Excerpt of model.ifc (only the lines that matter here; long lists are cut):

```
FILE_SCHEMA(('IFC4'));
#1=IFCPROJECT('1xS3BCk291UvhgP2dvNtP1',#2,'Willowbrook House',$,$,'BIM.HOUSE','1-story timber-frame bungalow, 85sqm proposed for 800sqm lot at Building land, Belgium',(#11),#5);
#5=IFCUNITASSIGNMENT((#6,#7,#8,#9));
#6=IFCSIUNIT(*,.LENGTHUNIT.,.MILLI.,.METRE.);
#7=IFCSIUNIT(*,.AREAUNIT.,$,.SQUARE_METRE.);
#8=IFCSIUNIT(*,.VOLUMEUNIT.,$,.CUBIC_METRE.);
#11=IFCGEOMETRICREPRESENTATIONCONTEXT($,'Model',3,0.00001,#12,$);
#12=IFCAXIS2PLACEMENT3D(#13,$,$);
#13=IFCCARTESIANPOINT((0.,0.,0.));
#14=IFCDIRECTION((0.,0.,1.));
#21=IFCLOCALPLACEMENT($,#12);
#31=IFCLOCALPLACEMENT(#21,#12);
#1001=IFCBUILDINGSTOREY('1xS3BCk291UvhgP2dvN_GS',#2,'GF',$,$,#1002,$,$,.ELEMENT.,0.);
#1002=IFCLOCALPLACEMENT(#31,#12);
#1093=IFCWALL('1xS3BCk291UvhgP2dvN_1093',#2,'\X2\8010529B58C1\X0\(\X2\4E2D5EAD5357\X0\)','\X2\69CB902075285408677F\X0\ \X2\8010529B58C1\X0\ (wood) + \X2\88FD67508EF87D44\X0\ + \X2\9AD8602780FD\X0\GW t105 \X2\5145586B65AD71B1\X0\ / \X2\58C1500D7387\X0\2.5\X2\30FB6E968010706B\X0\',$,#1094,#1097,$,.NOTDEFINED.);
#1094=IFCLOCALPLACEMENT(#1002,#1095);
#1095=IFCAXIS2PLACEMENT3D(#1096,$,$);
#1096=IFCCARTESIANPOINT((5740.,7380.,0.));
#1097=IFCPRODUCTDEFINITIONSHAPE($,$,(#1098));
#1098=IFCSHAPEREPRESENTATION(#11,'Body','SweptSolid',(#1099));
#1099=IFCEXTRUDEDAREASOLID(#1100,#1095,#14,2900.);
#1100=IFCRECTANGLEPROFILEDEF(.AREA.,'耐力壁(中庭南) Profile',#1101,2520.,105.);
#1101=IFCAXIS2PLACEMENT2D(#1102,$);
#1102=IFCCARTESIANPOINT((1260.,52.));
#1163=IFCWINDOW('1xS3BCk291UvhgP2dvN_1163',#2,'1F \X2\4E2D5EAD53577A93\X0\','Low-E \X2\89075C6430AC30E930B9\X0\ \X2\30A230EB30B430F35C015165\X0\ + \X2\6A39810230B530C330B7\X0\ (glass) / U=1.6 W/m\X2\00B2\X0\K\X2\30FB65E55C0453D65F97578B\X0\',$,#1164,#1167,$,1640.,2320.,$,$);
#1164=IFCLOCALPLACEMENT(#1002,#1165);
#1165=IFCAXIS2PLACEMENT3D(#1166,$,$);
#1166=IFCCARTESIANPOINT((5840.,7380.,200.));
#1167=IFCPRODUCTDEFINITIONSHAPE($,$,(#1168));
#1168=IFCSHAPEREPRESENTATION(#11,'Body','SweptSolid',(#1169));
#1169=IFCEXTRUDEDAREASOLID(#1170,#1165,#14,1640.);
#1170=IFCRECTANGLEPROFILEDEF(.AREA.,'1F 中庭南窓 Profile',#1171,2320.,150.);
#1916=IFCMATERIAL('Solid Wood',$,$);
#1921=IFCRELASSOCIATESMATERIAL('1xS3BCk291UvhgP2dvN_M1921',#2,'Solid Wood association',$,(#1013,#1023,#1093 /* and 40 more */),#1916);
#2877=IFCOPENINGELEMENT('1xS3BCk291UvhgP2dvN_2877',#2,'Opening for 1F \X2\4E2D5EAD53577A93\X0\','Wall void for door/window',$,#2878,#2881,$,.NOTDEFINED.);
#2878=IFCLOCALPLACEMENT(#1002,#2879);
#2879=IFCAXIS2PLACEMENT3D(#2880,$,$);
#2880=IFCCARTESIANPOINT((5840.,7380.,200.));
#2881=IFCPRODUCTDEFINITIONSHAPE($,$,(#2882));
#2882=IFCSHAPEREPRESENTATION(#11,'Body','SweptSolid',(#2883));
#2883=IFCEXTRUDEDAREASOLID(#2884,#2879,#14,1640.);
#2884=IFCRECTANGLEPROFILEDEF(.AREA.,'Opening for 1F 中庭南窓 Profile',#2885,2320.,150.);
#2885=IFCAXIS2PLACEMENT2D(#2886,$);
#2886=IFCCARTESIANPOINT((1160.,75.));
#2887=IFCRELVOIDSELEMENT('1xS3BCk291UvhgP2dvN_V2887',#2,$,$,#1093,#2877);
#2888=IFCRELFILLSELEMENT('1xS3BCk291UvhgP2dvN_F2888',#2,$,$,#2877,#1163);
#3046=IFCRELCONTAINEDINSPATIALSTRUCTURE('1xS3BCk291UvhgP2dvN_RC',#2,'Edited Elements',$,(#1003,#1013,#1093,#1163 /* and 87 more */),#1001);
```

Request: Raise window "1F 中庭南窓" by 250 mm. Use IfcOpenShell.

```python
import numpy as np
import ifcopenshell
import ifcopenshell.api.geometry
import ifcopenshell.util.placement
import ifcopenshell.util.unit

model = ifcopenshell.open("model.ifc")
unit_scale = ifcopenshell.util.unit.calculate_unit_scale(model)

window = model.by_guid("1xS3BCk291UvhgP2dvN_1163")
opening = window.FillsVoids[0].RelatingOpeningElement
dz = 0.25 / unit_scale

shift = np.array([0.0, 0.0, dz])
# The window is not placed relative to its opening, so move both.
for product in (opening, window):
    matrix = ifcopenshell.util.placement.get_local_placement(product.ObjectPlacement)
    matrix[:3, 3] += shift
    ifcopenshell.api.geometry.edit_object_placement(model, product=product, matrix=matrix, is_si=False)

print(f"moved by {dz * unit_scale:+.3f} m")

model.write("model-out.ifc")
```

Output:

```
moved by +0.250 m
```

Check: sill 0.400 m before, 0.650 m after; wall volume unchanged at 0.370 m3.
